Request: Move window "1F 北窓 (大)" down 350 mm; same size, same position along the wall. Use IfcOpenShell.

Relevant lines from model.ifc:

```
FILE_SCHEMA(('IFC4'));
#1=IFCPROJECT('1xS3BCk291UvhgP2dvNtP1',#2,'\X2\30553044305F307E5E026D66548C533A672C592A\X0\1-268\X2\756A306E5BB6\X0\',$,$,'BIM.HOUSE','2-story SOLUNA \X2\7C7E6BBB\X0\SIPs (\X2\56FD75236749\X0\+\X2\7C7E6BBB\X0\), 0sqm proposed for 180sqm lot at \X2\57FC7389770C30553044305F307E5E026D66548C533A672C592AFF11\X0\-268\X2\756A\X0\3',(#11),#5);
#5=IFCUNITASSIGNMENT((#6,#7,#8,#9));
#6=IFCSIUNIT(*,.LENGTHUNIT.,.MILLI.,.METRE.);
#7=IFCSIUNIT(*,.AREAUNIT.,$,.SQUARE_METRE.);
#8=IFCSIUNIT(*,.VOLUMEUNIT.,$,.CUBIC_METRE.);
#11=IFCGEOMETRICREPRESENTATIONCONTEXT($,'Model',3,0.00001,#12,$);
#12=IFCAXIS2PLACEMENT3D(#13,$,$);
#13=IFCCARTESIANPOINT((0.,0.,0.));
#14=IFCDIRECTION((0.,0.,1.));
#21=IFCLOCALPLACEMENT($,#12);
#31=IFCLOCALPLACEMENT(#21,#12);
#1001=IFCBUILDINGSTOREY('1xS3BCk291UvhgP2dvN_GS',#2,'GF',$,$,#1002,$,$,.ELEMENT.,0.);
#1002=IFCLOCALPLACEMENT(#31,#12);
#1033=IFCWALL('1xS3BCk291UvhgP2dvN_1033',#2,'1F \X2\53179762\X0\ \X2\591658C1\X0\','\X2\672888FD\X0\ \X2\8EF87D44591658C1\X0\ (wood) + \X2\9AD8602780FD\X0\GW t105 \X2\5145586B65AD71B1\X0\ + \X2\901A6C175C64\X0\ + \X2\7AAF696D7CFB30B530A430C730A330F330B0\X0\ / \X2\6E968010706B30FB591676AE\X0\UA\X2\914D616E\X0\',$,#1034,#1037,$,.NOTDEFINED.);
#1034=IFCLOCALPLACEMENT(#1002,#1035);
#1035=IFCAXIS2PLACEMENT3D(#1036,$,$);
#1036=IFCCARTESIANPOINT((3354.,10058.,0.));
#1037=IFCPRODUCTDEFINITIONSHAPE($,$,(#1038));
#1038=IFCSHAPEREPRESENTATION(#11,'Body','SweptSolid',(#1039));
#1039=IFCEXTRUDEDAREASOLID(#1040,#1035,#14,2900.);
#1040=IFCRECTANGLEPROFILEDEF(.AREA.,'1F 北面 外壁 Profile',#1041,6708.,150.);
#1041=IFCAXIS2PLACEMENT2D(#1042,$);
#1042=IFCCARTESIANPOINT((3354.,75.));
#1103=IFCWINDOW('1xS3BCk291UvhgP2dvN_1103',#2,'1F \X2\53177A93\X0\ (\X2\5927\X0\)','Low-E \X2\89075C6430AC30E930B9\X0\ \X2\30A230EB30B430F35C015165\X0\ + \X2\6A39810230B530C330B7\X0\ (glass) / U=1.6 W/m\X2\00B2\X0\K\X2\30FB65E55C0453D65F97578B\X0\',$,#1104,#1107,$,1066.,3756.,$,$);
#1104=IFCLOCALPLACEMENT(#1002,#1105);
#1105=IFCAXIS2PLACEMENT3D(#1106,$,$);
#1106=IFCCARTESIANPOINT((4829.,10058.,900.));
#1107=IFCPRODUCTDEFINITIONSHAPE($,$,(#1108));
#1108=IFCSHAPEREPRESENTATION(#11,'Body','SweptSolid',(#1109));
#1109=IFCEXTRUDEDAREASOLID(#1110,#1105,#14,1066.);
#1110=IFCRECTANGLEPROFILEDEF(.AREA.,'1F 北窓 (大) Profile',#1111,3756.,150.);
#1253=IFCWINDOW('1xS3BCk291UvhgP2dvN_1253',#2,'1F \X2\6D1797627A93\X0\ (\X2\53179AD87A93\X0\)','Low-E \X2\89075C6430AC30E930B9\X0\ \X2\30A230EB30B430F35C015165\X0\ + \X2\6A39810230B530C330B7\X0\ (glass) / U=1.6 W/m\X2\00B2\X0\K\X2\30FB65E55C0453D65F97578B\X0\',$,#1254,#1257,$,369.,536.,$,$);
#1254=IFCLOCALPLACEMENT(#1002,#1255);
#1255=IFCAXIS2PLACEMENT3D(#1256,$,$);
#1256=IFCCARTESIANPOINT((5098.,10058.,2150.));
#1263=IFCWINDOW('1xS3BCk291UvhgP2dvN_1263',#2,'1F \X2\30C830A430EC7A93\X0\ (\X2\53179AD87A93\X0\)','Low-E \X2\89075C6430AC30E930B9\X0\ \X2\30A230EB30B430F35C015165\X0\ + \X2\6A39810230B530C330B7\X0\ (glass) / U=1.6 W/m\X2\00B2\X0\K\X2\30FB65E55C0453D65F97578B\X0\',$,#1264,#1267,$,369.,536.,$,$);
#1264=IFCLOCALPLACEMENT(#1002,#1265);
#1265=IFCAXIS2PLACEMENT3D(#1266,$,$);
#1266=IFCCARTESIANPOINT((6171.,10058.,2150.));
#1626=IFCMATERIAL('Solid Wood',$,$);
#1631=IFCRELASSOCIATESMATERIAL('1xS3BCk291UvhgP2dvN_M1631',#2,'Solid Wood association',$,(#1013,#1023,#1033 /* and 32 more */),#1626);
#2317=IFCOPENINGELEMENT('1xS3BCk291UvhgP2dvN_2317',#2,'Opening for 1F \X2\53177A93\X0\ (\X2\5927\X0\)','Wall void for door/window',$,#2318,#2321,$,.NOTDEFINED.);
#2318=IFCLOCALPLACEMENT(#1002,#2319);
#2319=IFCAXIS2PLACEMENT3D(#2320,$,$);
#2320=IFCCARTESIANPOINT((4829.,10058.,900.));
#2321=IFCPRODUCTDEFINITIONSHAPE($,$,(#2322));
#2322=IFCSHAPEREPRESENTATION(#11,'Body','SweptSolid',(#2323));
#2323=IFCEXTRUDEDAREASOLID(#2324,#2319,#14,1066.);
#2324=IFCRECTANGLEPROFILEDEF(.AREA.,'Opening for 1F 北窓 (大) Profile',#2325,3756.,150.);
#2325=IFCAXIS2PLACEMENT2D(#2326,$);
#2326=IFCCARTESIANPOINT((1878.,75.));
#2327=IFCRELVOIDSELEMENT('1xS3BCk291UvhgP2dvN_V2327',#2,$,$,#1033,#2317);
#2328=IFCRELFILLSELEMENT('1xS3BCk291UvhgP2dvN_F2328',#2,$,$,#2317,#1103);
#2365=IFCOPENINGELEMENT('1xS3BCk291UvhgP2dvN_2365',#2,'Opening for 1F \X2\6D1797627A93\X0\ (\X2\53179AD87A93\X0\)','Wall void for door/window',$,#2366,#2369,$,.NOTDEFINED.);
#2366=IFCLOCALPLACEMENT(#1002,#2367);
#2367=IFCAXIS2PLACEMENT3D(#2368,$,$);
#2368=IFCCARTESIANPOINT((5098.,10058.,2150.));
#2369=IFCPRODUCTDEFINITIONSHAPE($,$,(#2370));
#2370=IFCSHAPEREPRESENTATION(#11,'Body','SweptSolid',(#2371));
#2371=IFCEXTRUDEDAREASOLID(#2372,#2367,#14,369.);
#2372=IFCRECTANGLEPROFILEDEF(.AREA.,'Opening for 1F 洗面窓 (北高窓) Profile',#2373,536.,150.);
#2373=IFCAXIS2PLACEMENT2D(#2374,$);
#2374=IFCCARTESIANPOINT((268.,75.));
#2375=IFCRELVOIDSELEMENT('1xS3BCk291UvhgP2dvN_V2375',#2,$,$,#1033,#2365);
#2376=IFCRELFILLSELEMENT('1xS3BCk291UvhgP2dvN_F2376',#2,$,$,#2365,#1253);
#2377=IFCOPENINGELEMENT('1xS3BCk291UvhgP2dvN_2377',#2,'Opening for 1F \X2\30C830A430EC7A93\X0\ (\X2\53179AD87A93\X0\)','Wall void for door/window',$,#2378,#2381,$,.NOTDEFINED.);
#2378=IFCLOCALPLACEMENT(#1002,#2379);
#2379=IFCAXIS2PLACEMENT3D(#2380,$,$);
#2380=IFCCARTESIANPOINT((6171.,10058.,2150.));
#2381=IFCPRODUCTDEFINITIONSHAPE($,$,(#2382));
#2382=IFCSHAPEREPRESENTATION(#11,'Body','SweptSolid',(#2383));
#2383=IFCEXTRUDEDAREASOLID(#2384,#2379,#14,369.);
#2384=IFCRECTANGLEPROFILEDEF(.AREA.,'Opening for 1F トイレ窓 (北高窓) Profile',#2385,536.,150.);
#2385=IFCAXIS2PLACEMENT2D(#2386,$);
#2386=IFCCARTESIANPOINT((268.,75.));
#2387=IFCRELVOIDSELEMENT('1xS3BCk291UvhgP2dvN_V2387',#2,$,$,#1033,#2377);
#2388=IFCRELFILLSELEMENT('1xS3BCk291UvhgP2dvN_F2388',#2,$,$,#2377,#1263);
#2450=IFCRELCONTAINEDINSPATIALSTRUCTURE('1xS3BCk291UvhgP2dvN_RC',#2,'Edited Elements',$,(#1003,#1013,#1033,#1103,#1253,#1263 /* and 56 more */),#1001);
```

```python
import numpy as np
import ifcopenshell
import ifcopenshell.api.geometry
import ifcopenshell.util.placement
import ifcopenshell.util.unit

model = ifcopenshell.open("model.ifc")
unit_scale = ifcopenshell.util.unit.calculate_unit_scale(model)

window = model.by_id(1103)
opening = window.FillsVoids[0].RelatingOpeningElement
dz = -0.35 / unit_scale

shift = np.array([0.0, 0.0, dz])
# The window is not placed relative to its opening, so move both.
for product in (opening, window):
    matrix = ifcopenshell.util.placement.get_local_placement(product.ObjectPlacement)
    matrix[:3, 3] += shift
    ifcopenshell.api.geometry.edit_object_placement(model, product=product, matrix=matrix, is_si=False)

print(f"moved by {dz * unit_scale:+.3f} m")

model.write("model_edited.ifc")
```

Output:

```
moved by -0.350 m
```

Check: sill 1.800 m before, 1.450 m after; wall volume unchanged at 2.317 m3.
